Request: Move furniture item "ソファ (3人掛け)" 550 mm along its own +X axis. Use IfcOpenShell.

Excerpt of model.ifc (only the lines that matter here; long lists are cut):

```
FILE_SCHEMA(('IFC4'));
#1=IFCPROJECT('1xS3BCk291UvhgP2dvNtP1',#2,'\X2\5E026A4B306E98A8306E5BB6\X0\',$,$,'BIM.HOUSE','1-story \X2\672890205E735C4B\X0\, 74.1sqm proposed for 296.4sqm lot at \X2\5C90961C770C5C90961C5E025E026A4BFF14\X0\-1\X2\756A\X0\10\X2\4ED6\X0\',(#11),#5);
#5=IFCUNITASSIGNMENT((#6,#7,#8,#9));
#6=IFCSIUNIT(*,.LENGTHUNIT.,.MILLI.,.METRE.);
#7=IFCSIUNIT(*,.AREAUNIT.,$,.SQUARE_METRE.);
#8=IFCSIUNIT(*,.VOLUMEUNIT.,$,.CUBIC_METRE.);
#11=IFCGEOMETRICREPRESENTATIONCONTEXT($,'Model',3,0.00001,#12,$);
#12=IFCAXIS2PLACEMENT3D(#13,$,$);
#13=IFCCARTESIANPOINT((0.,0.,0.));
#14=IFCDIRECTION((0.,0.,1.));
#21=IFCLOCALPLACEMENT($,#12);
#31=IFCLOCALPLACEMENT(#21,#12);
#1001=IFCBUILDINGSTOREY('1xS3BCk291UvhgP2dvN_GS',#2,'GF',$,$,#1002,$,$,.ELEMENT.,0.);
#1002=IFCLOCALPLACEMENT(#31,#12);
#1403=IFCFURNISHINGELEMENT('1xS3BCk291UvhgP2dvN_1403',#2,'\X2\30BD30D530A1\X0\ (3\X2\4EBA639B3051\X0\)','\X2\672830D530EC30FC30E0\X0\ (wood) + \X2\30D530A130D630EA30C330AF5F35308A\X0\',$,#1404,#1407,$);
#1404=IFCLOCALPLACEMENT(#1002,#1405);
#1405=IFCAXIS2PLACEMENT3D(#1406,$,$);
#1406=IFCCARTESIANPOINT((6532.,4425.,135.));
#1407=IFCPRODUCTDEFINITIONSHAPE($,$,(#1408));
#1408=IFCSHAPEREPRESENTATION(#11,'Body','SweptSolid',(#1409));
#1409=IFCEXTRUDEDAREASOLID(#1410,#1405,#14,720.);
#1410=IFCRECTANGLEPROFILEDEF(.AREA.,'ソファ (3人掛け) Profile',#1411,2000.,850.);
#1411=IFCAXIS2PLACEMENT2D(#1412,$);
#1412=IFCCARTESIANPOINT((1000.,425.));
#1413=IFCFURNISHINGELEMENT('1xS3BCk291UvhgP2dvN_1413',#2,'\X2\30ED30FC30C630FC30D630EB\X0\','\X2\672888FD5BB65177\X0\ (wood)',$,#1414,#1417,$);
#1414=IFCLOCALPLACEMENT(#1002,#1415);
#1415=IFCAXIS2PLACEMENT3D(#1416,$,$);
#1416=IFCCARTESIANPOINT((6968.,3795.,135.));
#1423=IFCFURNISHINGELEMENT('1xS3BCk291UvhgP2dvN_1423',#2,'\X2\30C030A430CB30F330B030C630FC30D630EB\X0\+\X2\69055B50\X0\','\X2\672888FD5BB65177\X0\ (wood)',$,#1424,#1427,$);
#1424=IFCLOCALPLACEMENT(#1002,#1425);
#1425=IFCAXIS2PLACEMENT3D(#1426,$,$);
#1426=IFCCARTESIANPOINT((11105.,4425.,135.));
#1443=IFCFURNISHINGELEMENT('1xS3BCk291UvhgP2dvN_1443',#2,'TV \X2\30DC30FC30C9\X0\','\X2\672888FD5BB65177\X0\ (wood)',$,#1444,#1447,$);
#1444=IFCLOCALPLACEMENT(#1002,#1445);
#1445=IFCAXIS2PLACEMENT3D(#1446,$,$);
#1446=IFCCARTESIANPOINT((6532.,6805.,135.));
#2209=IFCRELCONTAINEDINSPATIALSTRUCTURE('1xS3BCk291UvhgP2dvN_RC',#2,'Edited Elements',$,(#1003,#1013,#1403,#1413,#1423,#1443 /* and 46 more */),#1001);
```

```python
import ifcopenshell
import ifcopenshell.api.geometry
import ifcopenshell.util.placement
import ifcopenshell.util.unit

model = ifcopenshell.open("model.ifc")
unit_scale = ifcopenshell.util.unit.calculate_unit_scale(model)

item = model.by_guid("1xS3BCk291UvhgP2dvN_1403")
matrix = ifcopenshell.util.placement.get_local_placement(item.ObjectPlacement)
matrix[:3, 3] += matrix[:3, 0] * 0.55 / unit_scale
ifcopenshell.api.geometry.edit_object_placement(model, product=item, matrix=matrix, is_si=False)

print(ifcopenshell.util.placement.get_local_placement(item.ObjectPlacement).round(3) + 0.0)

model.write("model_v2.ifc")
```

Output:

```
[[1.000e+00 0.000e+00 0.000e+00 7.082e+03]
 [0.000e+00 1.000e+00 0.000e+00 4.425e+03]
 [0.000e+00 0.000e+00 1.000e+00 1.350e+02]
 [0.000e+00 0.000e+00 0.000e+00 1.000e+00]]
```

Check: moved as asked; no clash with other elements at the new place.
